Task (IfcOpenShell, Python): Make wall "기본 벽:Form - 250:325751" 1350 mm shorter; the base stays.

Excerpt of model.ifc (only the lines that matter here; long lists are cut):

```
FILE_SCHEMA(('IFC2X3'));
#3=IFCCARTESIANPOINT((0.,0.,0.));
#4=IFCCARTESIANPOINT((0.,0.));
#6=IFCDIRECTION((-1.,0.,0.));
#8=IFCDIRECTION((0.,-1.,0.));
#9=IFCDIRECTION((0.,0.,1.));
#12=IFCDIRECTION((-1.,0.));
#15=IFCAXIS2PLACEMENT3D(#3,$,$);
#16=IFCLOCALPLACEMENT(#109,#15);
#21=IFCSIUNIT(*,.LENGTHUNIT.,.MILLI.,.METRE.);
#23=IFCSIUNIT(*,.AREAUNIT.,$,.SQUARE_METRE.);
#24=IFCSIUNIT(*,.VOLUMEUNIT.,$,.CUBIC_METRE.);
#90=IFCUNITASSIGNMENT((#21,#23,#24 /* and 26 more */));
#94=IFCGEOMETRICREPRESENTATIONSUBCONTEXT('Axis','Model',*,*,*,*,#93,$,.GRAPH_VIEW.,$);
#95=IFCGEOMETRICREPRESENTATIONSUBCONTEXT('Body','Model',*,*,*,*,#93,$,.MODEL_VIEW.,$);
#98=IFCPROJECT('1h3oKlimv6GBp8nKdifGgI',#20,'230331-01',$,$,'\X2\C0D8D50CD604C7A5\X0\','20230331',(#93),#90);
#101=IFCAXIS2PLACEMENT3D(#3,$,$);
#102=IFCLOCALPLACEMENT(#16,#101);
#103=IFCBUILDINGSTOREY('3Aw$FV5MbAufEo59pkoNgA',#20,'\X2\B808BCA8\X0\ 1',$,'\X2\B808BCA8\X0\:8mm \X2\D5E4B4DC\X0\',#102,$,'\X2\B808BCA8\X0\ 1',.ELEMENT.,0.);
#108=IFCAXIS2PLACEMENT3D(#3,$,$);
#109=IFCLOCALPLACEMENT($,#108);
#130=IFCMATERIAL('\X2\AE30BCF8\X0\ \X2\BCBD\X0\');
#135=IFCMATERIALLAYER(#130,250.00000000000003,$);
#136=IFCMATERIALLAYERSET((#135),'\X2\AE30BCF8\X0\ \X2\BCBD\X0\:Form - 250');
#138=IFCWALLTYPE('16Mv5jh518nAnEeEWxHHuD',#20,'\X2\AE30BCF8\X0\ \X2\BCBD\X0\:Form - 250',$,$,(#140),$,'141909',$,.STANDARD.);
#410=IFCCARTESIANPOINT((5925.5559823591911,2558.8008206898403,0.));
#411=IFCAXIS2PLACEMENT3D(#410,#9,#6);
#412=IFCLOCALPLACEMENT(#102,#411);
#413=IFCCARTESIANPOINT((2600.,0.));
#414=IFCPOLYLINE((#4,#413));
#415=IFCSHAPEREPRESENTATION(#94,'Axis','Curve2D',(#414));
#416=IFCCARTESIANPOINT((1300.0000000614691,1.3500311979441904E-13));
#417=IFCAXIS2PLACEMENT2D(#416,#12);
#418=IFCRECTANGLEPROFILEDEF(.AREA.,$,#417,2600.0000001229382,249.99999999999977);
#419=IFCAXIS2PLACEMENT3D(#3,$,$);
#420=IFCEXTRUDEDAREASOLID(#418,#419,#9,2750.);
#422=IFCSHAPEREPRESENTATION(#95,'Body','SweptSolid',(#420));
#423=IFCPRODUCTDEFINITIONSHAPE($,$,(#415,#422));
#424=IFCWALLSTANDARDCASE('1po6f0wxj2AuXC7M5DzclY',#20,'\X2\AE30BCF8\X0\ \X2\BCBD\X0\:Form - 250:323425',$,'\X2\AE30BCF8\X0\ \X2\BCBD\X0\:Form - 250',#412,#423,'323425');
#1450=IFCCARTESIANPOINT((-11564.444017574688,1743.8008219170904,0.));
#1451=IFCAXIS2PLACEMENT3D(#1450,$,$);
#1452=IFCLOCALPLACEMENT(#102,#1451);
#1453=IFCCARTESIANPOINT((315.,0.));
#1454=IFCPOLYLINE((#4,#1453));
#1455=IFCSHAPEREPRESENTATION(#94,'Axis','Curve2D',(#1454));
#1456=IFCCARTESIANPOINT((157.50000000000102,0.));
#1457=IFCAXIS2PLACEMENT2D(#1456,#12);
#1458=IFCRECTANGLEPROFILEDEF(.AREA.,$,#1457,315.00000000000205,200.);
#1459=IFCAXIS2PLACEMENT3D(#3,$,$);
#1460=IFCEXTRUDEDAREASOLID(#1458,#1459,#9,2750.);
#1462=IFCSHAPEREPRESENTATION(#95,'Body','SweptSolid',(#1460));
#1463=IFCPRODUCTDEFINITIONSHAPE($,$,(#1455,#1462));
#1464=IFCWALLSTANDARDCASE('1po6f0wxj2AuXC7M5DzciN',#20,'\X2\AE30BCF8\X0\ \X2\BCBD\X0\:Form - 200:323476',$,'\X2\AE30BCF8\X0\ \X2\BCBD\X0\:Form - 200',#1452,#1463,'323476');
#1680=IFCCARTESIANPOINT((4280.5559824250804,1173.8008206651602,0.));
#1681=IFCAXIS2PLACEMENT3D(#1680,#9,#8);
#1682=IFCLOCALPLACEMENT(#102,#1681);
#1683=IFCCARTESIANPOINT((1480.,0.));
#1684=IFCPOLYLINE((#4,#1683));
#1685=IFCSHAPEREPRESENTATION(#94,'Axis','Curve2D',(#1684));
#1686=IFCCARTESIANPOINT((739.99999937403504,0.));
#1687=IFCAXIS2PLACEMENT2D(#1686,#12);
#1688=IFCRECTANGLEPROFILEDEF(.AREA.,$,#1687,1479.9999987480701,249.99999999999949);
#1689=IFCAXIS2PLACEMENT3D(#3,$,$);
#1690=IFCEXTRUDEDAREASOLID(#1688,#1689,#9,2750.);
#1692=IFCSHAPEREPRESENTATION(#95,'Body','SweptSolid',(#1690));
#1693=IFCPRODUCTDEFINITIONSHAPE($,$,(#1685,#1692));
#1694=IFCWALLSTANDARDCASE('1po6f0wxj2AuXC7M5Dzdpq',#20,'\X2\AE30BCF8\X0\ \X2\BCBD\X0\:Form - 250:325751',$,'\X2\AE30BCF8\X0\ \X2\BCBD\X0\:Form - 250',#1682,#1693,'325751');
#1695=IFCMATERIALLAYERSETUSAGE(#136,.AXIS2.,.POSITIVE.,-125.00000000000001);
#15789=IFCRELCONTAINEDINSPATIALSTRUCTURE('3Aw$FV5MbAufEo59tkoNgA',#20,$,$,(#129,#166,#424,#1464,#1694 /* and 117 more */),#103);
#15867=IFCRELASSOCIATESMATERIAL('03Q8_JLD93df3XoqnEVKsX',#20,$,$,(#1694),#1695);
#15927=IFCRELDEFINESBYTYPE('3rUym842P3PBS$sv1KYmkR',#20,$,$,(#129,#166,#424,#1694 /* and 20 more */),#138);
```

```python
import ifcopenshell
import ifcopenshell.geom
import ifcopenshell.util.representation
import ifcopenshell.util.shape
import ifcopenshell.util.unit

model = ifcopenshell.open("model.ifc")
unit_scale = ifcopenshell.util.unit.calculate_unit_scale(model)
settings = ifcopenshell.geom.settings()


def volume(element):
    """Net volume in cubic metres, openings subtracted."""
    shape = ifcopenshell.geom.create_shape(settings, element)
    return ifcopenshell.util.shape.get_volume(shape.geometry)


wall = model.by_guid("1po6f0wxj2AuXC7M5Dzdpq")
before = volume(wall)

body = ifcopenshell.util.representation.get_representation(wall, "Model", "Body")
solid = body.Items[0]
old_height = solid.Depth
solid.Depth -= 1.35 / unit_scale
after = volume(wall)

print(f"height {old_height:g} -> {solid.Depth:g}, volume {before:.3f} -> {after:.3f} m3")

model.write("model_v2.ifc")
```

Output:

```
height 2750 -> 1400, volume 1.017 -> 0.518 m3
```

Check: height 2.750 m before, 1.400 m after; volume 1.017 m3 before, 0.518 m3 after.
